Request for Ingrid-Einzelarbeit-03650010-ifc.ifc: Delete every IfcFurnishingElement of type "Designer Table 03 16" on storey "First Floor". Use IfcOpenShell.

First a look at what the model holds.

```python
import ifcopenshell
import ifcopenshell.util.element

model = ifcopenshell.open("Ingrid-Einzelarbeit-03650010-ifc.ifc")
print(model.schema)
storey = next(s for s in model.by_type("IfcBuildingStorey") if s.Name == "First Floor")
furniture = [e for e in ifcopenshell.util.element.get_decomposition(storey) if e.is_a("IfcFurnishingElement")]
seen = {}
for e in furniture:
    element_type = ifcopenshell.util.element.get_type(e)
    name = element_type.Name if element_type not in (None, e) else None
    seen[name] = seen.get(name, 0) + 1
for name, count in sorted(seen.items(), key=str):
    print(count, "x", name)
```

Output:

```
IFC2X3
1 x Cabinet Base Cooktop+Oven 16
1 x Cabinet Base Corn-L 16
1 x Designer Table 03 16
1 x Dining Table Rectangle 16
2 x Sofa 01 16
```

```python
import ifcopenshell
import ifcopenshell.api.root
import ifcopenshell.util.element

model = ifcopenshell.open("Ingrid-Einzelarbeit-03650010-ifc.ifc")

storey = next(s for s in model.by_type("IfcBuildingStorey") if s.Name == "First Floor")
furniture = [e for e in ifcopenshell.util.element.get_decomposition(storey) if e.is_a("IfcFurnishingElement")]
targets = [e for e in furniture if (t := ifcopenshell.util.element.get_type(e)) not in (None, e) and t.Name == "Designer Table 03 16"]

for e in targets:
    ifcopenshell.api.root.remove_product(model, product=e)
print(len(targets), "removed")

model.write("Ingrid-Einzelarbeit-03650010-ifc_edited.ifc")
```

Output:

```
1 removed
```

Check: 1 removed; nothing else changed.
